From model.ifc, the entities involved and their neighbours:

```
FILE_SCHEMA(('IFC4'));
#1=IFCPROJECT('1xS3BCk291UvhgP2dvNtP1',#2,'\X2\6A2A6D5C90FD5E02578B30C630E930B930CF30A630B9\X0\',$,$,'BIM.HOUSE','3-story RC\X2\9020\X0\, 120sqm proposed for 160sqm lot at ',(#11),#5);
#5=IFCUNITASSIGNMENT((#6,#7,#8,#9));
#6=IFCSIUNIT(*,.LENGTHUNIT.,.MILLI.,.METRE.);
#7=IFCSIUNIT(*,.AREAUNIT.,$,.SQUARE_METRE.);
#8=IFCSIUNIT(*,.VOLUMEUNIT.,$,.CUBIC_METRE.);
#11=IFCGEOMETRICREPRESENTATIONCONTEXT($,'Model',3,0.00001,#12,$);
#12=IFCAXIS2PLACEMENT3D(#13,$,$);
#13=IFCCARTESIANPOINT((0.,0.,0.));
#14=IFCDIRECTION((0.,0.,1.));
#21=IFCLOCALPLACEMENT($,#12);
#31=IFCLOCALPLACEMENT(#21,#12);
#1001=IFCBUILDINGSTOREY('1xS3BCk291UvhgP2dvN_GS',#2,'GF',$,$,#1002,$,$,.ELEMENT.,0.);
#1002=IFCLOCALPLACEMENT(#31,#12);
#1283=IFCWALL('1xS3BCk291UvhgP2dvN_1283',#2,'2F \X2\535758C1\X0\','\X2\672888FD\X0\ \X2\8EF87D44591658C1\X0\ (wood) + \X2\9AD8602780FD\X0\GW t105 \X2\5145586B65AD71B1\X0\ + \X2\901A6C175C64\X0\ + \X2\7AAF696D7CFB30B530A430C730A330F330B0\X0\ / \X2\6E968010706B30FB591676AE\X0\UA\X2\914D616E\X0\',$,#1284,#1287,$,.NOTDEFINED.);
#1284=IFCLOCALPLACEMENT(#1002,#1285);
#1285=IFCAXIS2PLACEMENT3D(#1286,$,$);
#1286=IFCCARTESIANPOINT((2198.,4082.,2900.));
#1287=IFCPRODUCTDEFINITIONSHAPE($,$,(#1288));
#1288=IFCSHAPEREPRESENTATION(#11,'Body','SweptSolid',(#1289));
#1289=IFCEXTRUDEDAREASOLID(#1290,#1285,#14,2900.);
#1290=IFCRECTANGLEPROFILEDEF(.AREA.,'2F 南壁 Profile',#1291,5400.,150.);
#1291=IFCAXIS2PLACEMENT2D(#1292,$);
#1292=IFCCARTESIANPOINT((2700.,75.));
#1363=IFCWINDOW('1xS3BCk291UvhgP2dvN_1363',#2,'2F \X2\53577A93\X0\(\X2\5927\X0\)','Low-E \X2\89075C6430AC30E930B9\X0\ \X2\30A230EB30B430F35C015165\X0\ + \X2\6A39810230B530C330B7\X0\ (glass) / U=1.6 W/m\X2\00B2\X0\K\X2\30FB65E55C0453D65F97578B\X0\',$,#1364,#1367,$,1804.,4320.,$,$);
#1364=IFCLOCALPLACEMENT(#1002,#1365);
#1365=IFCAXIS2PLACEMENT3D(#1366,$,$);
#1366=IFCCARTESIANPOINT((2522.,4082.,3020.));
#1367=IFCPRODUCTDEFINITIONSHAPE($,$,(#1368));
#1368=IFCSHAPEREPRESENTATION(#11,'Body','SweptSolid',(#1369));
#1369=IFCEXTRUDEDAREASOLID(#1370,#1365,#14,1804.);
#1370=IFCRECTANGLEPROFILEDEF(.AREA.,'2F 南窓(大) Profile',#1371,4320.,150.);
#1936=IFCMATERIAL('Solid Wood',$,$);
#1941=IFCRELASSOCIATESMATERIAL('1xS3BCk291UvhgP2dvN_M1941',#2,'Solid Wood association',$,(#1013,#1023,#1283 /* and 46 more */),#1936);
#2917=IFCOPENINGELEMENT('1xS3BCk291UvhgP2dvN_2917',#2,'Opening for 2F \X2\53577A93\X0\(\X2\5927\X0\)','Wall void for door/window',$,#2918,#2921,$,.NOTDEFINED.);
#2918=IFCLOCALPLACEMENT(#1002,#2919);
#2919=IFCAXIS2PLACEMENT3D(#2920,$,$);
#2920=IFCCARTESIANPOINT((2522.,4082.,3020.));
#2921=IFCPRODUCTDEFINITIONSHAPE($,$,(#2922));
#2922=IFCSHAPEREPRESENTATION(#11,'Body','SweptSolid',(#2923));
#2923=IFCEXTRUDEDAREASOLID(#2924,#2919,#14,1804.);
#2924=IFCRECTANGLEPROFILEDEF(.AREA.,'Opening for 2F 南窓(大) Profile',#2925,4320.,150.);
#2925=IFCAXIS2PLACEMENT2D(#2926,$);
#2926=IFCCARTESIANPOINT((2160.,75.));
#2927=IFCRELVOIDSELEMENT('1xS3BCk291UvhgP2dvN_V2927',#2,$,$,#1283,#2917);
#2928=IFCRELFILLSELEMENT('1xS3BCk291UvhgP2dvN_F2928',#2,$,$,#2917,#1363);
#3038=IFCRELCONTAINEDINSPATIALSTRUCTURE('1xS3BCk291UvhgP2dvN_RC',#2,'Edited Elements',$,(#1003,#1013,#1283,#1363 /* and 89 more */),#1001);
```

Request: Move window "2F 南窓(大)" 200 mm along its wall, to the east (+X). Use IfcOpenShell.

```python
import ifcopenshell
import ifcopenshell.api.geometry
import ifcopenshell.util.placement
import ifcopenshell.util.unit

model = ifcopenshell.open("model.ifc")
unit_scale = ifcopenshell.util.unit.calculate_unit_scale(model)

window = model.by_guid("1xS3BCk291UvhgP2dvN_1363")
opening = window.FillsVoids[0].RelatingOpeningElement
wall = opening.VoidsElements[0].RelatingBuildingElement

wall_matrix = ifcopenshell.util.placement.get_local_placement(wall.ObjectPlacement)
shift = wall_matrix[:3, 0] * 0.2 / unit_scale
before = ifcopenshell.util.placement.get_local_placement(window.ObjectPlacement)[:3, 3].copy()

# The window is not placed relative to its opening, so move both.
for product in (opening, window):
    matrix = ifcopenshell.util.placement.get_local_placement(product.ObjectPlacement)
    matrix[:3, 3] += shift
    ifcopenshell.api.geometry.edit_object_placement(model, product=product, matrix=matrix, is_si=False)

after = ifcopenshell.util.placement.get_local_placement(window.ObjectPlacement)[:3, 3]
print("window moved by", (after - before).round(3) + 0.0)

model.write("model_updated.ifc")
```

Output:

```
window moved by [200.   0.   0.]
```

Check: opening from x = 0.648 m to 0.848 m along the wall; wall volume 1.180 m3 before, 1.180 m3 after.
